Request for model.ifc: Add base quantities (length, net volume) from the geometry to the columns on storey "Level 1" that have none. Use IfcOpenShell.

First a look at what the model holds.

```python
import ifcopenshell
import ifcopenshell.util.element
import ifcopenshell.util.unit

model = ifcopenshell.open("model.ifc")
print(model.schema)
for unit_type in ("LENGTHUNIT", "AREAUNIT", "VOLUMEUNIT"):
    print(unit_type, ifcopenshell.util.unit.calculate_unit_scale(model, unit_type))
storey = next(s for s in model.by_type("IfcBuildingStorey") if s.Name == "Level 1")
columns = [e for e in ifcopenshell.util.element.get_decomposition(storey) if e.is_a("IfcColumn")]
for e in sorted(columns, key=lambda e: e.id()):
    print(e.id(), e.is_a(), e.Name, list(ifcopenshell.util.element.get_psets(e, qtos_only=True)), sep=" | ")
```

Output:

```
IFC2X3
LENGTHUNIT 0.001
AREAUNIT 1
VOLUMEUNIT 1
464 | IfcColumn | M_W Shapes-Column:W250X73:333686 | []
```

```python
import ifcopenshell
import ifcopenshell.api.pset
import ifcopenshell.geom
import ifcopenshell.util.element
import ifcopenshell.util.shape
import ifcopenshell.util.unit

model = ifcopenshell.open("model.ifc")
unit_scale = ifcopenshell.util.unit.calculate_unit_scale(model)
volume_scale = ifcopenshell.util.unit.calculate_unit_scale(model, "VOLUMEUNIT")
settings = ifcopenshell.geom.settings()

storey = next(s for s in model.by_type("IfcBuildingStorey") if s.Name == "Level 1")
columns = [e for e in ifcopenshell.util.element.get_decomposition(storey) if e.is_a("IfcColumn")]

for e in sorted(columns, key=lambda e: e.id()):
    if ifcopenshell.util.element.get_psets(e, qtos_only=True, should_inherit=False):
        continue
    # Geometry comes back in metres, in the element's own axes.
    shape = ifcopenshell.geom.create_shape(settings, e)
    values = {
        "Length": ifcopenshell.util.shape.get_z(shape.geometry) / unit_scale,
        "NetVolume": ifcopenshell.util.shape.get_volume(shape.geometry) / volume_scale,
    }
    qto = ifcopenshell.api.pset.add_qto(model, product=e, name="BaseQuantities")
    ifcopenshell.api.pset.edit_qto(model, qto=qto, properties=values)
    print(e.id(), {k: round(v, 3) for k, v in values.items()})

model.write("model_rev.ifc")
```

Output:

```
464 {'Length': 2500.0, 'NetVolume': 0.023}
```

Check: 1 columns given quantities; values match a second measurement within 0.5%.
